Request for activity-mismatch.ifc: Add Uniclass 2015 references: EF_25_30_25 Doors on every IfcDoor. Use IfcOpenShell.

First a look at what the model holds.

```python
import ifcopenshell

model = ifcopenshell.open("activity-mismatch.ifc")
print(model.schema)
print("classifications:", [c.Name for c in model.by_type("IfcClassification")])
for ifc_class in ("IfcDoor", "IfcRoof", "IfcStair", "IfcWall", "IfcWindow"):
    print(ifc_class, len(model.by_type(ifc_class)))
```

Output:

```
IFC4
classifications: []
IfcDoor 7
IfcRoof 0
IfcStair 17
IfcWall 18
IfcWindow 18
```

```python
import ifcopenshell
import ifcopenshell.api.classification

model = ifcopenshell.open("activity-mismatch.ifc")

system = ifcopenshell.api.classification.add_classification(model, classification="Uniclass 2015")

codes = {
    "IfcDoor": ("EF_25_30_25", "Doors"),
}
for ifc_class, (code, name) in codes.items():
    products = model.by_type(ifc_class)
    ifcopenshell.api.classification.add_reference(
        model, products=products, classification=system, identification=code, name=name
    )
    print(code, len(products))

model.write("activity-mismatch_v2.ifc")
```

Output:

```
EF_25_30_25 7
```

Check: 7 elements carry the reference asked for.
